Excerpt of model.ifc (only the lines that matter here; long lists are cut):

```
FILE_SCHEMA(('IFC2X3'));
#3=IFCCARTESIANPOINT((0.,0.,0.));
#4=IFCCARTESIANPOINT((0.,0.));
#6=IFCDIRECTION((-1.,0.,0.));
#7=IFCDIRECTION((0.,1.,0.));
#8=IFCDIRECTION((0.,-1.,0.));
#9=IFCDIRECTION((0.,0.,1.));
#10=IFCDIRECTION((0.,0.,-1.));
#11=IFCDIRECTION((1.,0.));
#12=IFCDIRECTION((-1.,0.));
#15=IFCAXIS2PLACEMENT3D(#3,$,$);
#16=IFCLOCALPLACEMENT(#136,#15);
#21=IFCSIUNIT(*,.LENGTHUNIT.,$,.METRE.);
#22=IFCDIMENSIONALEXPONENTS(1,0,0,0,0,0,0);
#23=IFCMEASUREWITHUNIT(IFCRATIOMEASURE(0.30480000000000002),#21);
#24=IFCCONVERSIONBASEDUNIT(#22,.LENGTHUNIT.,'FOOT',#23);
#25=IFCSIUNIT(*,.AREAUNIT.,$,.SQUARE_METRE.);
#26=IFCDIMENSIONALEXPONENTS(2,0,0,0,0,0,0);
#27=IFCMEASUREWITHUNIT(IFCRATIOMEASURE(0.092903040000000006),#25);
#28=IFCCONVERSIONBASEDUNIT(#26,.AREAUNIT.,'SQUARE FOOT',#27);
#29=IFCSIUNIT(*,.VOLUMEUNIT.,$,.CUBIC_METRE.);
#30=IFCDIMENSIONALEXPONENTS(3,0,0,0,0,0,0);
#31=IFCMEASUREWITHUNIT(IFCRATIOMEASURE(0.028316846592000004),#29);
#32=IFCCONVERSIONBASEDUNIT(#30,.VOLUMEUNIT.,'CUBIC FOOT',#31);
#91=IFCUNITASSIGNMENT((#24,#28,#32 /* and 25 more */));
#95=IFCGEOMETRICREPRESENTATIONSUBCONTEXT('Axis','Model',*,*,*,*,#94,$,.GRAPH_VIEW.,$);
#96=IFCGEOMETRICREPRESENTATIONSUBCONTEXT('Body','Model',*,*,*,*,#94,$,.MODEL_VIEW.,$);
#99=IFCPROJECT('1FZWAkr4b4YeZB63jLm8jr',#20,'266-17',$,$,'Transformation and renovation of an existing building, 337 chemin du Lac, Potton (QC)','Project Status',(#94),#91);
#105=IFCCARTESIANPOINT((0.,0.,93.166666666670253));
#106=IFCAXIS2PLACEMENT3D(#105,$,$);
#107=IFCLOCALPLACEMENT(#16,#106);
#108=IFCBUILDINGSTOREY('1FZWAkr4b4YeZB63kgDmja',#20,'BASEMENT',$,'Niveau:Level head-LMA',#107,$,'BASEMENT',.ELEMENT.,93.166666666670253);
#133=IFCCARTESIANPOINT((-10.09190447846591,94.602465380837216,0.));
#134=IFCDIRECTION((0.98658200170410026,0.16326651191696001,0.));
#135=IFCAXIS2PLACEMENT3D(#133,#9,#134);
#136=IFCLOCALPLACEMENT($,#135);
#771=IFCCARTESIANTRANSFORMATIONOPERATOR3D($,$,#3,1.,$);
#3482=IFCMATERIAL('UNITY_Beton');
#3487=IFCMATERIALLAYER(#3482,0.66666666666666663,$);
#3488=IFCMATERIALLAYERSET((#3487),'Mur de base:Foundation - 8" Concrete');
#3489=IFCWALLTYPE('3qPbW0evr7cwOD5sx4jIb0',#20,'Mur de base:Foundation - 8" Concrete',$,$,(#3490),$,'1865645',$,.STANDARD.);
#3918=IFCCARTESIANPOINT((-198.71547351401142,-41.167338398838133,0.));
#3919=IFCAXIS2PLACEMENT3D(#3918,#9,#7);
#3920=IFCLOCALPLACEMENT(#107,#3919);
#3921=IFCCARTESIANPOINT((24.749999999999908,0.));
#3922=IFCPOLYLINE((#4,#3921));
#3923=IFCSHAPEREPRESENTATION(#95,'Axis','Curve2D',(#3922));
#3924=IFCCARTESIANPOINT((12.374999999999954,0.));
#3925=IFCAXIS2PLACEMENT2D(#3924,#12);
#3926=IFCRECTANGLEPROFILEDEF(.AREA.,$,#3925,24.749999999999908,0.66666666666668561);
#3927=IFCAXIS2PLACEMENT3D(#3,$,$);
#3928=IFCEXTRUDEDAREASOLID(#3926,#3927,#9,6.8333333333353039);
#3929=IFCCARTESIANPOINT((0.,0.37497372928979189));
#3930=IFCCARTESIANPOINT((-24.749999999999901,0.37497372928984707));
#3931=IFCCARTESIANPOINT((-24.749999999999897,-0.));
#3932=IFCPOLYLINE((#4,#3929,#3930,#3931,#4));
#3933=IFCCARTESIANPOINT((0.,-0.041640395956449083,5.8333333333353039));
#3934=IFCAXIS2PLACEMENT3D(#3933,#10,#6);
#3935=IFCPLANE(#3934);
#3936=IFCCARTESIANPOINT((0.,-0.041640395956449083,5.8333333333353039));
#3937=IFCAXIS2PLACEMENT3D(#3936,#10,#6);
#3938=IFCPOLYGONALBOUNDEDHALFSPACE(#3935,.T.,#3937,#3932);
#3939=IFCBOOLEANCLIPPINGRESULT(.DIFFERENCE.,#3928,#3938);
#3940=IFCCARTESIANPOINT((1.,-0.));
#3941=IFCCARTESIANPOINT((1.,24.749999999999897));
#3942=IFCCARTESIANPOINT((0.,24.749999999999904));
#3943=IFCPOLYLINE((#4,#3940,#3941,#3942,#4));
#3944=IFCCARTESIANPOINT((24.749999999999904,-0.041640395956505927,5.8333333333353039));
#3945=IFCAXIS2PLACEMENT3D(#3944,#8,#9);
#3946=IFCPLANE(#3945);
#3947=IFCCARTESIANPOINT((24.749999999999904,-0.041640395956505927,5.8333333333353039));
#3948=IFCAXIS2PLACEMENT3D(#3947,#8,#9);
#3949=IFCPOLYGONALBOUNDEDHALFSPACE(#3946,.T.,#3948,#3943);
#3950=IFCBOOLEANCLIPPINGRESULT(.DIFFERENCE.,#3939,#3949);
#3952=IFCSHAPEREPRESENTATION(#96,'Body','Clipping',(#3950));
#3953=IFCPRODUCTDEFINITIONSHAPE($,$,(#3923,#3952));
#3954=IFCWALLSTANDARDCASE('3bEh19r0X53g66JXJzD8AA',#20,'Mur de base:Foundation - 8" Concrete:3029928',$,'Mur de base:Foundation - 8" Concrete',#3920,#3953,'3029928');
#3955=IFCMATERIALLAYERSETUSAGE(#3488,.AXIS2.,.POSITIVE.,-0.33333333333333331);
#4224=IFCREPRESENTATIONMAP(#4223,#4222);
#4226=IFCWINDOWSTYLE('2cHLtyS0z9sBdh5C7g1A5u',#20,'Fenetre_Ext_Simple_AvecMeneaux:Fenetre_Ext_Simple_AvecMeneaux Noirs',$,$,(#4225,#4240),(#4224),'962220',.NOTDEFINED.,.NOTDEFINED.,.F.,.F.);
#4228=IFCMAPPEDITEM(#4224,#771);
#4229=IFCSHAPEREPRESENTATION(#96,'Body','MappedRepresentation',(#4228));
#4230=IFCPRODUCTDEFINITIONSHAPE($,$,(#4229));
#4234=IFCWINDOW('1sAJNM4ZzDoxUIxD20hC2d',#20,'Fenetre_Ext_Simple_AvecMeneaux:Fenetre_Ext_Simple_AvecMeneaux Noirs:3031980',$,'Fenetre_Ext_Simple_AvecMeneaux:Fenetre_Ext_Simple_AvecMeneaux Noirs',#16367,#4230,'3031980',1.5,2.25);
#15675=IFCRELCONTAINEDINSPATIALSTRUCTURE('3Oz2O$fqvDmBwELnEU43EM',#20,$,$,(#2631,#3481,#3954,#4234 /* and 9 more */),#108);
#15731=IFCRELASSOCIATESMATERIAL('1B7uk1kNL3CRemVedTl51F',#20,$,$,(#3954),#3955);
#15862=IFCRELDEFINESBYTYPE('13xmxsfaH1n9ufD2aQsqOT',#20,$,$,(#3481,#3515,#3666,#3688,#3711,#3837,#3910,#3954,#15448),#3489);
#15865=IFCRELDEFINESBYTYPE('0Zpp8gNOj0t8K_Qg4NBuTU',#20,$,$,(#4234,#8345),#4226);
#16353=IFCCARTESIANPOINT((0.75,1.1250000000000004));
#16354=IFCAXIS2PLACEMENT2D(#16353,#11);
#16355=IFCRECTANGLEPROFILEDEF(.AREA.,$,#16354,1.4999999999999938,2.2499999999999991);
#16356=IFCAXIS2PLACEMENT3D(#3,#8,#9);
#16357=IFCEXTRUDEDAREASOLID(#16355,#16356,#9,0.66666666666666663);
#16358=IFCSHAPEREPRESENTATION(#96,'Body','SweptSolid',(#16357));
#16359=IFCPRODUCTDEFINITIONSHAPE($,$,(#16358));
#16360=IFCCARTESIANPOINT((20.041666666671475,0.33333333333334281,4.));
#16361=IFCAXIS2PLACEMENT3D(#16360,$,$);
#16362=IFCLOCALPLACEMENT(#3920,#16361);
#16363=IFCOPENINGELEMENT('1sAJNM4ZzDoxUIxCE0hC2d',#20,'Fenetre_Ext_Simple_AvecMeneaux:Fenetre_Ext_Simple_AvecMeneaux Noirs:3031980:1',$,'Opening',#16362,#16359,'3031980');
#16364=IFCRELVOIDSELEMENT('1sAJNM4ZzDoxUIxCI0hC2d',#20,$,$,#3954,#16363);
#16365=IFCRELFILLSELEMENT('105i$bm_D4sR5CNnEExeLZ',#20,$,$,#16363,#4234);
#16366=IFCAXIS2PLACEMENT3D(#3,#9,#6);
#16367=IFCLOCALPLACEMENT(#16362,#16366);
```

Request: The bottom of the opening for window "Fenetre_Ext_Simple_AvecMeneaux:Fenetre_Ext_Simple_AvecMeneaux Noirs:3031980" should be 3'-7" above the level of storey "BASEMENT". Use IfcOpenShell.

```python
import numpy as np
import ifcopenshell
import ifcopenshell.api.geometry
import ifcopenshell.geom
import ifcopenshell.util.element
import ifcopenshell.util.placement
import ifcopenshell.util.shape
import ifcopenshell.util.unit

model = ifcopenshell.open("model.ifc")
unit_scale = ifcopenshell.util.unit.calculate_unit_scale(model)

window = model.by_guid("1sAJNM4ZzDoxUIxD20hC2d")
opening = window.FillsVoids[0].RelatingOpeningElement
storey = ifcopenshell.util.element.get_container(window, ifc_class="IfcBuildingStorey")
level = ifcopenshell.util.placement.get_local_placement(storey.ObjectPlacement)[2, 3]

# The opening's origin need not be at the sill, so measure its lowest point.
shape = ifcopenshell.geom.create_shape(ifcopenshell.geom.settings(), opening)
bottom = ifcopenshell.util.shape.get_shape_bottom_elevation(shape, shape.geometry) / unit_scale
dz = level + 43 * 0.0254 / unit_scale - bottom

shift = np.array([0.0, 0.0, dz])
# The window is placed relative to its opening, so it follows when the opening moves.
matrix = ifcopenshell.util.placement.get_local_placement(opening.ObjectPlacement)
matrix[:3, 3] += shift
ifcopenshell.api.geometry.edit_object_placement(
    model, product=opening, matrix=matrix, is_si=False, should_transform_children=True
)

print(f"moved by {dz * unit_scale:+.3f} m")

model.write("model_updated.ifc")
```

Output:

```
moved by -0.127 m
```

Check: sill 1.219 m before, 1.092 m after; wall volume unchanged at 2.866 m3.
